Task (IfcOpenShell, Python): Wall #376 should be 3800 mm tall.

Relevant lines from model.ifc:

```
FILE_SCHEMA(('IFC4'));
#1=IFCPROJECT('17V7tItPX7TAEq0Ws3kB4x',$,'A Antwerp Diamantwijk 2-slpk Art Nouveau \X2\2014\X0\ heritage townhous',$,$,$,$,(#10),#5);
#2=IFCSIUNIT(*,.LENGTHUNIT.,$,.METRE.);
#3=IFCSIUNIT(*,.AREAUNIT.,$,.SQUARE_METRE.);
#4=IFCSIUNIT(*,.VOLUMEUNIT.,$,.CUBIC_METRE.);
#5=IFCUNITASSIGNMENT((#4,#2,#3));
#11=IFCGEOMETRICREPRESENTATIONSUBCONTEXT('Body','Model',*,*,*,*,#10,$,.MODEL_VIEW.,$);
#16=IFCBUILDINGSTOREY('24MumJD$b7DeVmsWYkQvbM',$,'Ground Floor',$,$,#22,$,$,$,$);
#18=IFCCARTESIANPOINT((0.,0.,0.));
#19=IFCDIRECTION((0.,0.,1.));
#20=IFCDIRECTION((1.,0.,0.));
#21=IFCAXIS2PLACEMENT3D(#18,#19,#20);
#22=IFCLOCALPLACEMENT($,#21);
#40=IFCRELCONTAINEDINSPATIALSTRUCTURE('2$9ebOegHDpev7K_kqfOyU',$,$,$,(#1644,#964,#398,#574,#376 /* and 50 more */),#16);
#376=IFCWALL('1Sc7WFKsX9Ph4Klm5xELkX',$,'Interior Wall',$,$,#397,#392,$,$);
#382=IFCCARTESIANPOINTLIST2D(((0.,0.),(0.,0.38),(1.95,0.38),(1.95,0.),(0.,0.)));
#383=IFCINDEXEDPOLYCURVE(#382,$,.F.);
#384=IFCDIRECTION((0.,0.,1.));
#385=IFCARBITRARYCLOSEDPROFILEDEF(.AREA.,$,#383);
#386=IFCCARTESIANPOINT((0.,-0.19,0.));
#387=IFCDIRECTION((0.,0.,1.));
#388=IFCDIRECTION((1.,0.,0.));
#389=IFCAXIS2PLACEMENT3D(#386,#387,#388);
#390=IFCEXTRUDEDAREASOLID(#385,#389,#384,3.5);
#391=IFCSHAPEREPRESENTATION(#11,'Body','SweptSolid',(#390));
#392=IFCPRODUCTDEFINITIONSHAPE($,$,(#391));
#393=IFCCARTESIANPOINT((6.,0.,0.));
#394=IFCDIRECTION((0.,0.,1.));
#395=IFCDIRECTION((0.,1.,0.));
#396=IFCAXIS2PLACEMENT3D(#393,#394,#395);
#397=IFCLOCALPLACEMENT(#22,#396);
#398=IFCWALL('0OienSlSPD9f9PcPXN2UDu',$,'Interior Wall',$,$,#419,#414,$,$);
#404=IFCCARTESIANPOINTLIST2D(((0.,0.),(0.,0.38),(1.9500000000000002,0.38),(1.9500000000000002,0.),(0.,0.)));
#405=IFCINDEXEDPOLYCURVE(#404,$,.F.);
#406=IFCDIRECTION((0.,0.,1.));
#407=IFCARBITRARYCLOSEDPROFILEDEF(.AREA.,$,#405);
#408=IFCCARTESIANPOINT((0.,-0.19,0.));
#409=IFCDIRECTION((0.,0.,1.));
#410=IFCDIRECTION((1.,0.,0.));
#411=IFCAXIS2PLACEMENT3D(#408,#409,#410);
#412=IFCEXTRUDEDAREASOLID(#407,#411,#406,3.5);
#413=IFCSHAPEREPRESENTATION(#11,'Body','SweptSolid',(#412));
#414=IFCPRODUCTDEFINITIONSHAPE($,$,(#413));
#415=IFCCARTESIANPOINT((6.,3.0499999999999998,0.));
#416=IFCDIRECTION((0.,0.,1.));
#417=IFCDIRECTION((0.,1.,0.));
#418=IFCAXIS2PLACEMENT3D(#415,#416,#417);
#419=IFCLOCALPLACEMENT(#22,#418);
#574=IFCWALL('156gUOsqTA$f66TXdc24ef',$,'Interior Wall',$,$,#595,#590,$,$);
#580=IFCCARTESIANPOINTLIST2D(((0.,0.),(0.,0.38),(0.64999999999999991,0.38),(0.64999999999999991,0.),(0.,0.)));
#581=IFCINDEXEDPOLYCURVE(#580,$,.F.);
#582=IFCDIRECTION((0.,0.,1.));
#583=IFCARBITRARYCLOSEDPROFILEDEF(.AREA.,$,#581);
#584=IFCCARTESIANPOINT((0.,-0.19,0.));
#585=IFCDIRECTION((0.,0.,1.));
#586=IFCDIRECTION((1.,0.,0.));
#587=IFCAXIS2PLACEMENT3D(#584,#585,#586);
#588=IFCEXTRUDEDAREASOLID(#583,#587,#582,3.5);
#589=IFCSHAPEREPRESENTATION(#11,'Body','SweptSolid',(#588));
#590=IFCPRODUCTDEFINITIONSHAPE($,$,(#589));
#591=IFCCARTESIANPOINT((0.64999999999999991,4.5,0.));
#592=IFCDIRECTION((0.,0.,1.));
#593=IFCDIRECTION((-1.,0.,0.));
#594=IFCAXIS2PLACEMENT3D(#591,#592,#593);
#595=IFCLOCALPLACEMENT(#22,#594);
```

```python
import ifcopenshell
import ifcopenshell.geom
import ifcopenshell.util.representation
import ifcopenshell.util.shape
import ifcopenshell.util.unit

model = ifcopenshell.open("model.ifc")
unit_scale = ifcopenshell.util.unit.calculate_unit_scale(model)
settings = ifcopenshell.geom.settings()


def volume(element):
    """Net volume in cubic metres, openings subtracted."""
    shape = ifcopenshell.geom.create_shape(settings, element)
    return ifcopenshell.util.shape.get_volume(shape.geometry)


wall = model.by_guid("1Sc7WFKsX9Ph4Klm5xELkX")
before = volume(wall)

body = ifcopenshell.util.representation.get_representation(wall, "Model", "Body")
solid = body.Items[0]
old_height = solid.Depth
solid.Depth = 3.8 / unit_scale
after = volume(wall)

print(f"height {old_height:g} -> {solid.Depth:g}, volume {before:.3f} -> {after:.3f} m3")

model.write("model_edited.ifc")
```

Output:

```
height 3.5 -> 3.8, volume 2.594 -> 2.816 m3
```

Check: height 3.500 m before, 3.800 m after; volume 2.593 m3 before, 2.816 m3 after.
